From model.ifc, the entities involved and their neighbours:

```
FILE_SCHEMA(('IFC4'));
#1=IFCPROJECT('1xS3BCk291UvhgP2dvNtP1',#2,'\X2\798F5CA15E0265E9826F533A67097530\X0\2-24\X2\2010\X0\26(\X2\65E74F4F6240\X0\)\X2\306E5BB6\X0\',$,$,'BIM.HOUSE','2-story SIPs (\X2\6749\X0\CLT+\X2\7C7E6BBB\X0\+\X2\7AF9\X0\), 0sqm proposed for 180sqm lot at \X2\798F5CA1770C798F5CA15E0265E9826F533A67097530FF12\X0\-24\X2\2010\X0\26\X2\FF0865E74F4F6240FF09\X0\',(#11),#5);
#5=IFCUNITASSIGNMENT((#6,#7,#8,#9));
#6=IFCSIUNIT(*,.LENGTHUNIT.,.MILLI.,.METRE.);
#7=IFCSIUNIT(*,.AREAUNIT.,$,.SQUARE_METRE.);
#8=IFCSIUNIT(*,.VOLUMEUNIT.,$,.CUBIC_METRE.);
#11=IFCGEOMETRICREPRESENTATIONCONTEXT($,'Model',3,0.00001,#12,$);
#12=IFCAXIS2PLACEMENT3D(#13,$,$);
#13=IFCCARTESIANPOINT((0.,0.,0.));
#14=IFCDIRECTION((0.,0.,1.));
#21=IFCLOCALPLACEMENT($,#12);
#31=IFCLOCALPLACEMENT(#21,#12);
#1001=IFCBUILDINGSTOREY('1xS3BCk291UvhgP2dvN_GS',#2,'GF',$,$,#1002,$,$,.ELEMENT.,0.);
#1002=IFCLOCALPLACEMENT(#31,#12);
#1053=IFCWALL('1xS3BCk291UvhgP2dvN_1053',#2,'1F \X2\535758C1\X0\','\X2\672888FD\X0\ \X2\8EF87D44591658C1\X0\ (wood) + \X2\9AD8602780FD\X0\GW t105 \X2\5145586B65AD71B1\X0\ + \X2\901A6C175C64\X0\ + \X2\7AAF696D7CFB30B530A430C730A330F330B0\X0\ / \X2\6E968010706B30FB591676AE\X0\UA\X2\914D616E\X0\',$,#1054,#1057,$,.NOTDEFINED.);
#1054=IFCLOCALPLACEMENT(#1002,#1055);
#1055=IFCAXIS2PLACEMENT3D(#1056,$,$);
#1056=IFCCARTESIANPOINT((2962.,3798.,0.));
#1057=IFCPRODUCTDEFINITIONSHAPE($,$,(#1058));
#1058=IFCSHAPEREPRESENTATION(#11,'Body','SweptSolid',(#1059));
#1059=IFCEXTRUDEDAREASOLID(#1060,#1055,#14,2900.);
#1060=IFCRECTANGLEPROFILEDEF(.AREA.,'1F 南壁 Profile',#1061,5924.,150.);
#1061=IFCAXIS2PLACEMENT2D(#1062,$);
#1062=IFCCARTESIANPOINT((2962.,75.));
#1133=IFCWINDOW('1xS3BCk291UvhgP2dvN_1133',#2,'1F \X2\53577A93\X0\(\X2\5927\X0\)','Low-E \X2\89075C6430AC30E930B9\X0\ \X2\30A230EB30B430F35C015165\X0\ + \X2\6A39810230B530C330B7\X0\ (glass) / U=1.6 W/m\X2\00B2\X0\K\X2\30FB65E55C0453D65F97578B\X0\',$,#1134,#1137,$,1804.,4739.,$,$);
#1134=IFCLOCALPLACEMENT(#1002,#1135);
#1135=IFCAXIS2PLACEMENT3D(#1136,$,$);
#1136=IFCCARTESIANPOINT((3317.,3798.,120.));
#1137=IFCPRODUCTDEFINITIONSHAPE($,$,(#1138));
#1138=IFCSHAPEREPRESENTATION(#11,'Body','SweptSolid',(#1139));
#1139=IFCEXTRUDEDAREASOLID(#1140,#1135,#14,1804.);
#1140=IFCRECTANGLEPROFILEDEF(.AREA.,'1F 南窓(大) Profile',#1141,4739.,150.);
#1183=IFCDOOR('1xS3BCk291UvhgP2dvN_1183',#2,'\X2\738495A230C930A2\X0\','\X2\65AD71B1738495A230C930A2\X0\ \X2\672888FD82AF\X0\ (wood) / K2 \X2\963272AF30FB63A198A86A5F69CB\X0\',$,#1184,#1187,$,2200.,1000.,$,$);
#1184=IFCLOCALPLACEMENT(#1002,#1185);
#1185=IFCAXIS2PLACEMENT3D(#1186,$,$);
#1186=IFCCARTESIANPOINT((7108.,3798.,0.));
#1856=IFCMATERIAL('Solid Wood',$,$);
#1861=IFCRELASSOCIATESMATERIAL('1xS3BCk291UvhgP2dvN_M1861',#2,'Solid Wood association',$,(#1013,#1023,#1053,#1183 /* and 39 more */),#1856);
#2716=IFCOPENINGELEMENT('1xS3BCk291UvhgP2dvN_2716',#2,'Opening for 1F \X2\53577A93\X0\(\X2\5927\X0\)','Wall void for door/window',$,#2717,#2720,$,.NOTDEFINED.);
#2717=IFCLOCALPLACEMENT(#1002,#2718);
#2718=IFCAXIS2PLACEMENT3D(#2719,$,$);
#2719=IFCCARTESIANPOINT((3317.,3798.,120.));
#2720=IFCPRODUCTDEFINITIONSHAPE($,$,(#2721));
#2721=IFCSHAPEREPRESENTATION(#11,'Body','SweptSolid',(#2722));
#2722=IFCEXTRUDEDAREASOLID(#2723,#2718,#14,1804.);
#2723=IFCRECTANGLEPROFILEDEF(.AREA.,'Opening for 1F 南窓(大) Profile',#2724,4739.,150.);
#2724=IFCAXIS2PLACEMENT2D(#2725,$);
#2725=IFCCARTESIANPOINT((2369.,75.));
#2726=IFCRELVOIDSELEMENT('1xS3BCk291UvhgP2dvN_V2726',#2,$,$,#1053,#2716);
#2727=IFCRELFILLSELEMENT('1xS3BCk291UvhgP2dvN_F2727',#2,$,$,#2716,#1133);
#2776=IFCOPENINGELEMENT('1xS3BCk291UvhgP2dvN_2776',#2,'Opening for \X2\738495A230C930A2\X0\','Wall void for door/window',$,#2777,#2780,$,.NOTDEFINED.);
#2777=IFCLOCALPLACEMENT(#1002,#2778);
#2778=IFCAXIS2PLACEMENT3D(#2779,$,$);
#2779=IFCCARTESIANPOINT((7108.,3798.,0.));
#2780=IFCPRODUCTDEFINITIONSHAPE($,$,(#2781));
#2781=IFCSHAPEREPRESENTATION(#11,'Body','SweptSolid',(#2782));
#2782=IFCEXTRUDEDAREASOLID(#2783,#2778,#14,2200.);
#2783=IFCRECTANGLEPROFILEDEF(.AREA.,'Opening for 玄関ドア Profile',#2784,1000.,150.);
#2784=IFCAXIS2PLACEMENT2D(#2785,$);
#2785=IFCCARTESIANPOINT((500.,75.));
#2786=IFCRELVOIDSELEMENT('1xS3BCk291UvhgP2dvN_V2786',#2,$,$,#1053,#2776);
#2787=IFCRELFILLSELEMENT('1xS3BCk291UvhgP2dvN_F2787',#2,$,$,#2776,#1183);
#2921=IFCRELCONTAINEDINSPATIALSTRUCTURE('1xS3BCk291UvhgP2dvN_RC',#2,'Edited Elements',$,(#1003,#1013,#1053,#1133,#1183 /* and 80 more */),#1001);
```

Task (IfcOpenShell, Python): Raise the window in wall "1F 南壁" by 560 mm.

```python
import numpy as np
import ifcopenshell
import ifcopenshell.api.geometry
import ifcopenshell.util.placement
import ifcopenshell.util.unit

model = ifcopenshell.open("model.ifc")
unit_scale = ifcopenshell.util.unit.calculate_unit_scale(model)

window = model.by_id(1133)
opening = window.FillsVoids[0].RelatingOpeningElement
dz = 0.56 / unit_scale

shift = np.array([0.0, 0.0, dz])
# The window is not placed relative to its opening, so move both.
for product in (opening, window):
    matrix = ifcopenshell.util.placement.get_local_placement(product.ObjectPlacement)
    matrix[:3, 3] += shift
    ifcopenshell.api.geometry.edit_object_placement(model, product=product, matrix=matrix, is_si=False)

print(f"moved by {dz * unit_scale:+.3f} m")

model.write("model_updated.ifc")
```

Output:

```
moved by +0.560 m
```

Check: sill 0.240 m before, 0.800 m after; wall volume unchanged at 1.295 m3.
